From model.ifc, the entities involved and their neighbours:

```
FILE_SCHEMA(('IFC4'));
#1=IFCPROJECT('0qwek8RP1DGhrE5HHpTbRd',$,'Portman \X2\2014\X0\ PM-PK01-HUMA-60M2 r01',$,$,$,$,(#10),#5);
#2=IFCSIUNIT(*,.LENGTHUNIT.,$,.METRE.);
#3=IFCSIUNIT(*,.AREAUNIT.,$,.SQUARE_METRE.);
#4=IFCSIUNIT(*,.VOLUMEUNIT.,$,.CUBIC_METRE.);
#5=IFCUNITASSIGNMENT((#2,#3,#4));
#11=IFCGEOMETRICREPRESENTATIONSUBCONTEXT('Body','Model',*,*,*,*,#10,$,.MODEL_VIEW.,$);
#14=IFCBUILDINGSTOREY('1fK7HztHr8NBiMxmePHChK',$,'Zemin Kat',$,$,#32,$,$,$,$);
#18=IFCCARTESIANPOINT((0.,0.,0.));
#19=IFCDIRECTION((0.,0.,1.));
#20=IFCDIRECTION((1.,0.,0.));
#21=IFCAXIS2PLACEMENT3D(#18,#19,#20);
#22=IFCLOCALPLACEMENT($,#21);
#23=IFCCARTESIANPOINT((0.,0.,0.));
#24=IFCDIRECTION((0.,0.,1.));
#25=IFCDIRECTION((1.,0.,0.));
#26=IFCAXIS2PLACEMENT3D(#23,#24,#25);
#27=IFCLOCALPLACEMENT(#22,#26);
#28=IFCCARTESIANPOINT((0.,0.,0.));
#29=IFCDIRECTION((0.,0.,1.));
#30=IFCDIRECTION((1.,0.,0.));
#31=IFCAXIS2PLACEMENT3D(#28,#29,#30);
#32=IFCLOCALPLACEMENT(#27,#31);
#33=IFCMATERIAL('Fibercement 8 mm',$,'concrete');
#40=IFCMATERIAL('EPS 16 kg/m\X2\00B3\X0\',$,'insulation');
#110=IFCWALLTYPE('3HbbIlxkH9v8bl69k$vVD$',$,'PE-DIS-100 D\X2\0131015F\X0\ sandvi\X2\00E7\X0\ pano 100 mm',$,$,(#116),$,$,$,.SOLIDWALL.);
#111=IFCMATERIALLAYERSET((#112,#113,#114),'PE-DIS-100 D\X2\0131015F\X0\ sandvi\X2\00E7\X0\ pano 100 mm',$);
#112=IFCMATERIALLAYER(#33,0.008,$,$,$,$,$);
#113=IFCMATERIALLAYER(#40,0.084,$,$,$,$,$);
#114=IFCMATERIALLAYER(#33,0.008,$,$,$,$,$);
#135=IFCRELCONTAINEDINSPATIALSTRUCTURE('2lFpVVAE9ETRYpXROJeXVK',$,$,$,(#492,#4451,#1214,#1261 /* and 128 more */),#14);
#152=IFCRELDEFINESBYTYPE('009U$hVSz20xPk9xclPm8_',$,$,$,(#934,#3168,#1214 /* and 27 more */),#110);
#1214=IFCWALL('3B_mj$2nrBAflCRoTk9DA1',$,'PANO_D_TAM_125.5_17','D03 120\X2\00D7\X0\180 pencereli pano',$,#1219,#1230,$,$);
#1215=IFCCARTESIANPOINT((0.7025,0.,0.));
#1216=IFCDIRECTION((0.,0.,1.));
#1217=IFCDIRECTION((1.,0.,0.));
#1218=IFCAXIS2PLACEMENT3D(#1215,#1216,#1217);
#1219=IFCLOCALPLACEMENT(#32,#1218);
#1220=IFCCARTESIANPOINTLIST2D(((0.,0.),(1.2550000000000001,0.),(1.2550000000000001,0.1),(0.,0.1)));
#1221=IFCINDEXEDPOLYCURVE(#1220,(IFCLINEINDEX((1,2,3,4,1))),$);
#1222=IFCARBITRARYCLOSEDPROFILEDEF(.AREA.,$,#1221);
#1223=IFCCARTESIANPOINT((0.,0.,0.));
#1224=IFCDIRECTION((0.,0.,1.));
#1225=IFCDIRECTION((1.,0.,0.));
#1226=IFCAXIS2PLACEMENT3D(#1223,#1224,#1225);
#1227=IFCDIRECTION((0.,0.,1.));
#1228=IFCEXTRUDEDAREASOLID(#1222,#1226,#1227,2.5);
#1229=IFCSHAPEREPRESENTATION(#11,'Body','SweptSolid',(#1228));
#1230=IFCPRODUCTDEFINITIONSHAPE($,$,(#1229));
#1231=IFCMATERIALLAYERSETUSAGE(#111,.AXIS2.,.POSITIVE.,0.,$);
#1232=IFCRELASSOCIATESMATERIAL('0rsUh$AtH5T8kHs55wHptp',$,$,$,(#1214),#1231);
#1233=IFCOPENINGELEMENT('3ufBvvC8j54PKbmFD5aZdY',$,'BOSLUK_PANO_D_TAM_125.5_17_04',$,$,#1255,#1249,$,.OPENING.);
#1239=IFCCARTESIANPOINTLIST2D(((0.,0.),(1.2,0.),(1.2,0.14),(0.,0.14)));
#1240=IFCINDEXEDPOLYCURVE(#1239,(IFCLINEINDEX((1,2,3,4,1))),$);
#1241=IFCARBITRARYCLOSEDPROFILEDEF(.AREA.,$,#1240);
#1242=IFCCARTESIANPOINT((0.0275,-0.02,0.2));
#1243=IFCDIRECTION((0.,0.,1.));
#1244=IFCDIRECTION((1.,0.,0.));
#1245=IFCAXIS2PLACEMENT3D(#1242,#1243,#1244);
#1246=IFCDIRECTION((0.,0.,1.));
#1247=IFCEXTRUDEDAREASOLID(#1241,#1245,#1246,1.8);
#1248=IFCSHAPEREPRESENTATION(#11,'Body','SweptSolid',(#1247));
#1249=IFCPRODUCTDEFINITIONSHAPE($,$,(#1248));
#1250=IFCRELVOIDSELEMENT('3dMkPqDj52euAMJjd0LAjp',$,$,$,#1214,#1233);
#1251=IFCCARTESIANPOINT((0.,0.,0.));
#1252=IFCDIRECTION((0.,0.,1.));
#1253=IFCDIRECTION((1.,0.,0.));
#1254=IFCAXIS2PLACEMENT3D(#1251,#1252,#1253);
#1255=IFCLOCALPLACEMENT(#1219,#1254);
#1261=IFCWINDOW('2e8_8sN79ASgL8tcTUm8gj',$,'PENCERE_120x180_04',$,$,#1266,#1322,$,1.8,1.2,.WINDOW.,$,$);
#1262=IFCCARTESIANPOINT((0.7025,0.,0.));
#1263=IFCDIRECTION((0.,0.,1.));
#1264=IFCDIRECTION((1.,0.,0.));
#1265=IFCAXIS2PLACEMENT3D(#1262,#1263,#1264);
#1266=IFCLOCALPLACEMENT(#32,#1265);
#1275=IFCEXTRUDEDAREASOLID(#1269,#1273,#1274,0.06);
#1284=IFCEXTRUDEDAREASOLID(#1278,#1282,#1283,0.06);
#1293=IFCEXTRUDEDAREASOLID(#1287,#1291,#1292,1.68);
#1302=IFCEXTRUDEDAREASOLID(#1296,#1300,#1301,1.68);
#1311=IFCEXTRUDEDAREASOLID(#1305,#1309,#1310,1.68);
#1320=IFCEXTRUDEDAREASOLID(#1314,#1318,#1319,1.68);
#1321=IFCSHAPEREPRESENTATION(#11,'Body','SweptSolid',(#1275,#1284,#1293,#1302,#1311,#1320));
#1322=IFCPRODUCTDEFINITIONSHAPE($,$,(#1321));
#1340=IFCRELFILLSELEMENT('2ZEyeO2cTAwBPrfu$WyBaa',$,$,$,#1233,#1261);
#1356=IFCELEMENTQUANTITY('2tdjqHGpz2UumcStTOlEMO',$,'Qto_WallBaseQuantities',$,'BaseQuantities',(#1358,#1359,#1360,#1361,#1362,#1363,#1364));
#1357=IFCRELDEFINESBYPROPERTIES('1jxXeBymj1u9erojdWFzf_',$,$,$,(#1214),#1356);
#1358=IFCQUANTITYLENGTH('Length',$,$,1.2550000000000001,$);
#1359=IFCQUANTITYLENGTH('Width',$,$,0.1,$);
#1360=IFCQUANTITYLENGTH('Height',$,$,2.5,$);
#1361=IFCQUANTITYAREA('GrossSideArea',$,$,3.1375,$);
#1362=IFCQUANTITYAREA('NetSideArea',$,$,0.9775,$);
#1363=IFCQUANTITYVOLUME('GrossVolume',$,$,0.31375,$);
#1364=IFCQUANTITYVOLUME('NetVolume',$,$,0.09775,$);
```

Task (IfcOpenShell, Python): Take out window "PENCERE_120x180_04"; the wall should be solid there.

```python
import ifcopenshell
import ifcopenshell.api.feature
import ifcopenshell.api.pset
import ifcopenshell.api.root
import ifcopenshell.geom
import ifcopenshell.util.element
import ifcopenshell.util.shape
import ifcopenshell.util.unit

model = ifcopenshell.open("model.ifc")
area_scale = ifcopenshell.util.unit.calculate_unit_scale(model, "AREAUNIT")
volume_scale = ifcopenshell.util.unit.calculate_unit_scale(model, "VOLUMEUNIT")
settings = ifcopenshell.geom.settings()


def volume(element):
    """Net volume in cubic metres, openings subtracted."""
    shape = ifcopenshell.geom.create_shape(settings, element)
    return ifcopenshell.util.shape.get_volume(shape.geometry)


window = model.by_guid("2e8_8sN79ASgL8tcTUm8gj")
opening = window.FillsVoids[0].RelatingOpeningElement
wall = opening.VoidsElements[0].RelatingBuildingElement
before = volume(wall)

ifcopenshell.api.root.remove_product(model, product=window)
ifcopenshell.api.feature.remove_feature(model, feature=opening)

after = volume(wall)
thickness = 0.1  # wall thickness in metres

# Update the wall's stored quantities.
qto = model.by_id(ifcopenshell.util.element.get_pset(wall, "Qto_WallBaseQuantities", should_inherit=False)["id"])
ifcopenshell.api.pset.edit_qto(model, qto=qto, properties={
    "NetSideArea": after / thickness / area_scale,
    "NetVolume": after / volume_scale,
})

print(f"wall volume {before:.3f} -> {after:.3f} m3")

model.write("model_v2.ifc")
```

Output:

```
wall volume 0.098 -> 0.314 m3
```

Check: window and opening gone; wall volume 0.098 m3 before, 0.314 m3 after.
